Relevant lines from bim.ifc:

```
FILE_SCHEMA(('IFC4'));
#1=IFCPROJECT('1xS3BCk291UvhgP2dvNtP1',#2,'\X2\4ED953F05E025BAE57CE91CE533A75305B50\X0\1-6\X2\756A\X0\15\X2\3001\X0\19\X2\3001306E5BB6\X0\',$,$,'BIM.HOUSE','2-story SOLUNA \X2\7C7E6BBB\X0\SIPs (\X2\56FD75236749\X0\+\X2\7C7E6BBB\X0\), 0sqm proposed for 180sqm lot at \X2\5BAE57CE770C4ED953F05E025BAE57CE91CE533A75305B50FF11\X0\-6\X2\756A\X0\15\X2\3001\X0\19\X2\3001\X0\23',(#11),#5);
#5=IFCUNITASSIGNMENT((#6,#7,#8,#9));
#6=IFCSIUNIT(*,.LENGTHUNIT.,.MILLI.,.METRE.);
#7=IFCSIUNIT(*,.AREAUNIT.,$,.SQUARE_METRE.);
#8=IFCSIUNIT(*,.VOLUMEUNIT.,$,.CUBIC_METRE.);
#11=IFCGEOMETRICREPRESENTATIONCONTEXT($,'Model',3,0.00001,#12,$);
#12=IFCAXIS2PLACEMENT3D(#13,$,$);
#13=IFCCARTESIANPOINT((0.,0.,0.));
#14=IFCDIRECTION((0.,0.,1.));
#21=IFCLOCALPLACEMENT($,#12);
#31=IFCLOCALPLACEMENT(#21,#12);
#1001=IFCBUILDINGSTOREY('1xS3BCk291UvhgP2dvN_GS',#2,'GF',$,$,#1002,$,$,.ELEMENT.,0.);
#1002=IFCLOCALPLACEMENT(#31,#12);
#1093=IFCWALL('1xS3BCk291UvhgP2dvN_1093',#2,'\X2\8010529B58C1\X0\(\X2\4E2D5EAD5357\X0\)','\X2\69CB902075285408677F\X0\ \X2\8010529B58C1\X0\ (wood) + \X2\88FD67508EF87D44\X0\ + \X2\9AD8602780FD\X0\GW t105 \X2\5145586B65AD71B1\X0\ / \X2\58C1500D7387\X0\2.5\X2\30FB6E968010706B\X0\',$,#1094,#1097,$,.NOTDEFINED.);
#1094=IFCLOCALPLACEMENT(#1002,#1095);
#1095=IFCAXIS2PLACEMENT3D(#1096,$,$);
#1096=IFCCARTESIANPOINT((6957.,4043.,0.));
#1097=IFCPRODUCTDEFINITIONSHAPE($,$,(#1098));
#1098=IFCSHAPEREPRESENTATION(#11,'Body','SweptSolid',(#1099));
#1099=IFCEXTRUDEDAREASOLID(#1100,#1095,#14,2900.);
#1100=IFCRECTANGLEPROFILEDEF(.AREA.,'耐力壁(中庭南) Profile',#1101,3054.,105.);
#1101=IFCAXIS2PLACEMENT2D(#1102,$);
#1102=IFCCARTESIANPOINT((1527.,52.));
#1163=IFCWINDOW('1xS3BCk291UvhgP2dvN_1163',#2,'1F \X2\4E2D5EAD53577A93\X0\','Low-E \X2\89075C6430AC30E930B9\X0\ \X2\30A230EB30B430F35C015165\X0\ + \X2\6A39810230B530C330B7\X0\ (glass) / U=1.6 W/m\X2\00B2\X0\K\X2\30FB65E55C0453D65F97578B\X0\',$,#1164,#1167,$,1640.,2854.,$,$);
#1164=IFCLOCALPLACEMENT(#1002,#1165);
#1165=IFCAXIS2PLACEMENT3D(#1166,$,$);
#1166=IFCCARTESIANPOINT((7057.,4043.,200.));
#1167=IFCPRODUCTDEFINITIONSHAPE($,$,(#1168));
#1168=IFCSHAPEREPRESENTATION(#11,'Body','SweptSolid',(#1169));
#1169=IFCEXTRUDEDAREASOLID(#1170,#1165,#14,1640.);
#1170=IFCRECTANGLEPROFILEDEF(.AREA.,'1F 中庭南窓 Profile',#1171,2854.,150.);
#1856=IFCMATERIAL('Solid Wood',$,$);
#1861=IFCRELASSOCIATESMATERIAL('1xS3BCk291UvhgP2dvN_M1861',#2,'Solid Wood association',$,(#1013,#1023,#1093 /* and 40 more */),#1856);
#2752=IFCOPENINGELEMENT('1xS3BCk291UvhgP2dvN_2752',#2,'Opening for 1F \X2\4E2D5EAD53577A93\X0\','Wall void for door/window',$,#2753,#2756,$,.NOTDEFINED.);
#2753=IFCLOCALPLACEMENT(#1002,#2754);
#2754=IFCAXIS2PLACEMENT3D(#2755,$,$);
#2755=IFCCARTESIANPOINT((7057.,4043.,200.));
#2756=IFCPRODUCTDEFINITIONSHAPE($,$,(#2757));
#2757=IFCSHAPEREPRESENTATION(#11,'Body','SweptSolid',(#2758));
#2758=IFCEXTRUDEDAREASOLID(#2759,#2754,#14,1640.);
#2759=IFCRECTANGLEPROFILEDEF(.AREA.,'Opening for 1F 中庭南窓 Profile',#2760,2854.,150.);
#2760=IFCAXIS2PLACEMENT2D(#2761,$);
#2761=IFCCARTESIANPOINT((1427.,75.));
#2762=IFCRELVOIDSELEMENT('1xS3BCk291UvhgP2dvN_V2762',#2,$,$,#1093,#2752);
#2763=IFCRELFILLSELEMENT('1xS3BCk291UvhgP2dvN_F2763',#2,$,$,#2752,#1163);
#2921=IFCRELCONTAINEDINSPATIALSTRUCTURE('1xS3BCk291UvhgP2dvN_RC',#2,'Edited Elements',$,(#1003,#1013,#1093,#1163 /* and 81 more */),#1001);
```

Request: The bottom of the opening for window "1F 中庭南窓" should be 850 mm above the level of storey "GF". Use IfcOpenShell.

```python
import numpy as np
import ifcopenshell
import ifcopenshell.api.geometry
import ifcopenshell.geom
import ifcopenshell.util.element
import ifcopenshell.util.placement
import ifcopenshell.util.shape
import ifcopenshell.util.unit

model = ifcopenshell.open("bim.ifc")
unit_scale = ifcopenshell.util.unit.calculate_unit_scale(model)

window = model.by_guid("1xS3BCk291UvhgP2dvN_1163")
opening = window.FillsVoids[0].RelatingOpeningElement
storey = ifcopenshell.util.element.get_container(window, ifc_class="IfcBuildingStorey")
level = ifcopenshell.util.placement.get_local_placement(storey.ObjectPlacement)[2, 3]

# The opening's origin need not be at the sill, so measure its lowest point.
shape = ifcopenshell.geom.create_shape(ifcopenshell.geom.settings(), opening)
bottom = ifcopenshell.util.shape.get_shape_bottom_elevation(shape, shape.geometry) / unit_scale
dz = level + 850.0 - bottom

shift = np.array([0.0, 0.0, dz])
# The window is not placed relative to its opening, so move both.
for product in (opening, window):
    matrix = ifcopenshell.util.placement.get_local_placement(product.ObjectPlacement)
    matrix[:3, 3] += shift
    ifcopenshell.api.geometry.edit_object_placement(model, product=product, matrix=matrix, is_si=False)

print(f"moved by {dz * unit_scale:+.3f} m")

model.write("bim_edited.ifc")
```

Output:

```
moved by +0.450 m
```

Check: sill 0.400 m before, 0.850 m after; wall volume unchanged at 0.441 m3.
